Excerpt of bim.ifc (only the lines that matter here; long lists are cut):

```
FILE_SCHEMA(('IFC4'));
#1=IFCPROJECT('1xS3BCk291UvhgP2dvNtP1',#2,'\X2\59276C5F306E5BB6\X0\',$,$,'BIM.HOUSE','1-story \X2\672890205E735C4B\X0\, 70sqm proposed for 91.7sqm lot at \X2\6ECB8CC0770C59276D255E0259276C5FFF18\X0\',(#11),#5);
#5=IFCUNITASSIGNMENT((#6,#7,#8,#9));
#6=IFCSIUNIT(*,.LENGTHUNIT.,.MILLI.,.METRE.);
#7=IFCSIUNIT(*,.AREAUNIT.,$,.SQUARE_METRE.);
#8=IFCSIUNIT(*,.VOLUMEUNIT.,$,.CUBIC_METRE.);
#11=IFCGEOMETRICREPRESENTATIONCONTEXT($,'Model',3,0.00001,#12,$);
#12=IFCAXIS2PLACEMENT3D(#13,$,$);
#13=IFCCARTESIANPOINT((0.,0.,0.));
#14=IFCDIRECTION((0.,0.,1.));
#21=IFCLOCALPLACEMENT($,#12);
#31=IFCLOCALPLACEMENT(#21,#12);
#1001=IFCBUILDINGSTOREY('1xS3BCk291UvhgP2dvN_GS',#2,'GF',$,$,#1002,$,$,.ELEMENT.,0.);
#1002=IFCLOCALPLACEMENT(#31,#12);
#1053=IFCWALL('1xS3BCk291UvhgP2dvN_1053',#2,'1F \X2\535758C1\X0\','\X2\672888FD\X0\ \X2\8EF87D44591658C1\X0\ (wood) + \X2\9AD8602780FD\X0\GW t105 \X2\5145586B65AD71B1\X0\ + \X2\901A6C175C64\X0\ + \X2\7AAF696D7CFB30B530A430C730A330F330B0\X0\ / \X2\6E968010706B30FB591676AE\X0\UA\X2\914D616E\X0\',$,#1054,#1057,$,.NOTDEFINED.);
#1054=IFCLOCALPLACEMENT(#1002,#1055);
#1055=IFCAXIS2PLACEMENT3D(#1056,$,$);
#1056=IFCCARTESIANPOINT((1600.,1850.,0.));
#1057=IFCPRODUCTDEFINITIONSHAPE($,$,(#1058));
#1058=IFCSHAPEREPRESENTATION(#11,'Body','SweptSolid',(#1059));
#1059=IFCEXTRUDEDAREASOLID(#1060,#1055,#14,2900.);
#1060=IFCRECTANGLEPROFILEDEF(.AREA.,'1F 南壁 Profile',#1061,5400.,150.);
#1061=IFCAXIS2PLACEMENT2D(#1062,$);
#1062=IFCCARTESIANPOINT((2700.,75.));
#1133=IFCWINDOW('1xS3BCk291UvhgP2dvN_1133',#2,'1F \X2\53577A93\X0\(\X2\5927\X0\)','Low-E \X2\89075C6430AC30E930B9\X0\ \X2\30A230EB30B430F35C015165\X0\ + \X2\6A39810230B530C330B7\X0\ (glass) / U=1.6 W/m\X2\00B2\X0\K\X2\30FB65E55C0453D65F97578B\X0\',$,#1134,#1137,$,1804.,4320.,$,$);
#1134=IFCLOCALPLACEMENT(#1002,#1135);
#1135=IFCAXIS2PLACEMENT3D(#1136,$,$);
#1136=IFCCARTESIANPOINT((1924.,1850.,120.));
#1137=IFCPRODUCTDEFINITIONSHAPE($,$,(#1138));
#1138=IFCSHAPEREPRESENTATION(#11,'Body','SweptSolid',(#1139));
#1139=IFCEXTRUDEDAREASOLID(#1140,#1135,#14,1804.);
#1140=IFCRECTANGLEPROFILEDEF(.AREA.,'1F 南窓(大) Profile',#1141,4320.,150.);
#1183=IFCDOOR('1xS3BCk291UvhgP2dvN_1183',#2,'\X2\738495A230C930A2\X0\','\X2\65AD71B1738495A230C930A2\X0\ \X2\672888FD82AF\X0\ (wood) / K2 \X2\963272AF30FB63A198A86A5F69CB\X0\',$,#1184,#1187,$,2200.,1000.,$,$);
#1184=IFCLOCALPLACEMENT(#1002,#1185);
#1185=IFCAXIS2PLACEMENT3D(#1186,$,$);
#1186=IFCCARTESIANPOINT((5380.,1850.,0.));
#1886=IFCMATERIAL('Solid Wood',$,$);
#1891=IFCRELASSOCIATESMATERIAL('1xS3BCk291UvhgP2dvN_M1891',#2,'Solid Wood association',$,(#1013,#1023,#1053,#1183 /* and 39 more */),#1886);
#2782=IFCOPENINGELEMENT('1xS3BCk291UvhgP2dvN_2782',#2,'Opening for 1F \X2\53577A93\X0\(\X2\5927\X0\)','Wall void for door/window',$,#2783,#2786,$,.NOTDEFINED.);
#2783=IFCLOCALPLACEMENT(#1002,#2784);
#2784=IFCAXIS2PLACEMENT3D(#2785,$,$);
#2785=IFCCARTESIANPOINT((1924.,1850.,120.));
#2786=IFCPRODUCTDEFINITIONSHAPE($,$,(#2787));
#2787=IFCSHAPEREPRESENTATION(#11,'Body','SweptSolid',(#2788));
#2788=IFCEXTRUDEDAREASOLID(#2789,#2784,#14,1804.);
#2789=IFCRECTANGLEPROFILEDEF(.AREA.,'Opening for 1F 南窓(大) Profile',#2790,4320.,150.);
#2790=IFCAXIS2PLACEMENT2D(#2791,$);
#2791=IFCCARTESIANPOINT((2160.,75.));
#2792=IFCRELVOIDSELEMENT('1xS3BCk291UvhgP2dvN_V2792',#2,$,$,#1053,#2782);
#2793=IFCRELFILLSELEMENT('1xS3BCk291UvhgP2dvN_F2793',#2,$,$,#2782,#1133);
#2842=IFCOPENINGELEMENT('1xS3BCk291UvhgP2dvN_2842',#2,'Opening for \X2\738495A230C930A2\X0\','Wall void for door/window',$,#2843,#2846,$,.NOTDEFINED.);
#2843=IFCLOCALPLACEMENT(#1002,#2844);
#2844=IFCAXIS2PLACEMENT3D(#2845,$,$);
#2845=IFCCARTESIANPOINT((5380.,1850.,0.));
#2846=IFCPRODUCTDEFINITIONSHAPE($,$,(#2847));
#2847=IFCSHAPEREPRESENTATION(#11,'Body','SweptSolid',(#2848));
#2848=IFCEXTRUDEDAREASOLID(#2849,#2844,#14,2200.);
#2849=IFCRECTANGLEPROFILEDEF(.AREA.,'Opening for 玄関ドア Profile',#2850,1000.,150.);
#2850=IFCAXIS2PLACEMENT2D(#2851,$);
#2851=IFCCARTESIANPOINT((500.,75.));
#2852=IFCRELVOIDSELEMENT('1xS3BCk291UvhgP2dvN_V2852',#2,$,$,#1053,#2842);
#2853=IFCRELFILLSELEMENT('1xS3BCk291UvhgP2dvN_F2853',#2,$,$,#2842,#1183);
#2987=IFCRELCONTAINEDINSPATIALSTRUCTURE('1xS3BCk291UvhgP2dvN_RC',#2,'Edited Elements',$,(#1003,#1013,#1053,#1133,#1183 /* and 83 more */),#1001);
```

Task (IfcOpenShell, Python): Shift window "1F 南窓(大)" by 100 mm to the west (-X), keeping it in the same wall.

```python
import ifcopenshell
import ifcopenshell.api.geometry
import ifcopenshell.util.placement

model = ifcopenshell.open("bim.ifc")

window = model.by_guid("1xS3BCk291UvhgP2dvN_1133")
opening = window.FillsVoids[0].RelatingOpeningElement
wall = opening.VoidsElements[0].RelatingBuildingElement

wall_matrix = ifcopenshell.util.placement.get_local_placement(wall.ObjectPlacement)
shift = wall_matrix[:3, 0] * -100.0
before = ifcopenshell.util.placement.get_local_placement(window.ObjectPlacement)[:3, 3].copy()

# The window is not placed relative to its opening, so move both.
for product in (opening, window):
    matrix = ifcopenshell.util.placement.get_local_placement(product.ObjectPlacement)
    matrix[:3, 3] += shift
    ifcopenshell.api.geometry.edit_object_placement(model, product=product, matrix=matrix, is_si=False)

after = ifcopenshell.util.placement.get_local_placement(window.ObjectPlacement)[:3, 3]
print("window moved by", (after - before).round(3) + 0.0)

model.write("bim_v2.ifc")
```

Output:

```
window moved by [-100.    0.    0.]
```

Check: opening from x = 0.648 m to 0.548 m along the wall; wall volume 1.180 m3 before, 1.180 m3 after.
